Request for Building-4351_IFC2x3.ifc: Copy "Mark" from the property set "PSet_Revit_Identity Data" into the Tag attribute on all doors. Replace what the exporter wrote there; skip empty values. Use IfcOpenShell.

First a look at what the model holds.

```python
import ifcopenshell
import ifcopenshell.util.element

model = ifcopenshell.open("Building-4351_IFC2x3.ifc")
print(model.schema)
doors = model.by_type("IfcDoor")
print(len(doors), "doors")
for e in doors[:8]:
    source = ifcopenshell.util.element.get_pset(e, "PSet_Revit_Identity Data", "Mark")
    target = e.Tag
    print(e.id(), repr(source), repr(target), sep=" | ")
```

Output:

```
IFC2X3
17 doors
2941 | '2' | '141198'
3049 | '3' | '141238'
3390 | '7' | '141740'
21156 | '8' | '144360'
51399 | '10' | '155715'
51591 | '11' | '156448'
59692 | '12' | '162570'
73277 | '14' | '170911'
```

```python
import ifcopenshell
import ifcopenshell.util.element

model = ifcopenshell.open("Building-4351_IFC2x3.ifc")

count = 0
for e in model.by_type("IfcDoor"):
    value = ifcopenshell.util.element.get_pset(e, "PSet_Revit_Identity Data", "Mark")
    current = e.Tag
    if not value or not value.strip() or current == value:
        continue
    e.Tag = value
    count += 1

print(count, "doors updated")

model.write("Building-4351_IFC2x3_rev.ifc")
```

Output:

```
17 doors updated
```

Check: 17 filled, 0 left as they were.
